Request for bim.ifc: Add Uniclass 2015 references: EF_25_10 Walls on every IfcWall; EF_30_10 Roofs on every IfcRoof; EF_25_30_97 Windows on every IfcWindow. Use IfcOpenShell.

First a look at what the model holds.

```python
import ifcopenshell

model = ifcopenshell.open("bim.ifc")
print(model.schema)
print("classifications:", [c.Name for c in model.by_type("IfcClassification")])
for ifc_class in ("IfcDoor", "IfcRoof", "IfcStair", "IfcWall", "IfcWindow"):
    print(ifc_class, len(model.by_type(ifc_class)))
```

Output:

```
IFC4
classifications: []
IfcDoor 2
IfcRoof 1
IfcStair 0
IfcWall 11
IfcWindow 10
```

```python
import ifcopenshell
import ifcopenshell.api.classification

model = ifcopenshell.open("bim.ifc")

system = ifcopenshell.api.classification.add_classification(model, classification="Uniclass 2015")

codes = {
    "IfcWall": ("EF_25_10", "Walls"),
    "IfcRoof": ("EF_30_10", "Roofs"),
    "IfcWindow": ("EF_25_30_97", "Windows"),
}
for ifc_class, (code, name) in codes.items():
    products = model.by_type(ifc_class)
    ifcopenshell.api.classification.add_reference(
        model, products=products, classification=system, identification=code, name=name
    )
    print(code, len(products))

model.write("bim_updated.ifc")
```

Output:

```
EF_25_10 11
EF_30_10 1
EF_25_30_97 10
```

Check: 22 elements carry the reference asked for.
